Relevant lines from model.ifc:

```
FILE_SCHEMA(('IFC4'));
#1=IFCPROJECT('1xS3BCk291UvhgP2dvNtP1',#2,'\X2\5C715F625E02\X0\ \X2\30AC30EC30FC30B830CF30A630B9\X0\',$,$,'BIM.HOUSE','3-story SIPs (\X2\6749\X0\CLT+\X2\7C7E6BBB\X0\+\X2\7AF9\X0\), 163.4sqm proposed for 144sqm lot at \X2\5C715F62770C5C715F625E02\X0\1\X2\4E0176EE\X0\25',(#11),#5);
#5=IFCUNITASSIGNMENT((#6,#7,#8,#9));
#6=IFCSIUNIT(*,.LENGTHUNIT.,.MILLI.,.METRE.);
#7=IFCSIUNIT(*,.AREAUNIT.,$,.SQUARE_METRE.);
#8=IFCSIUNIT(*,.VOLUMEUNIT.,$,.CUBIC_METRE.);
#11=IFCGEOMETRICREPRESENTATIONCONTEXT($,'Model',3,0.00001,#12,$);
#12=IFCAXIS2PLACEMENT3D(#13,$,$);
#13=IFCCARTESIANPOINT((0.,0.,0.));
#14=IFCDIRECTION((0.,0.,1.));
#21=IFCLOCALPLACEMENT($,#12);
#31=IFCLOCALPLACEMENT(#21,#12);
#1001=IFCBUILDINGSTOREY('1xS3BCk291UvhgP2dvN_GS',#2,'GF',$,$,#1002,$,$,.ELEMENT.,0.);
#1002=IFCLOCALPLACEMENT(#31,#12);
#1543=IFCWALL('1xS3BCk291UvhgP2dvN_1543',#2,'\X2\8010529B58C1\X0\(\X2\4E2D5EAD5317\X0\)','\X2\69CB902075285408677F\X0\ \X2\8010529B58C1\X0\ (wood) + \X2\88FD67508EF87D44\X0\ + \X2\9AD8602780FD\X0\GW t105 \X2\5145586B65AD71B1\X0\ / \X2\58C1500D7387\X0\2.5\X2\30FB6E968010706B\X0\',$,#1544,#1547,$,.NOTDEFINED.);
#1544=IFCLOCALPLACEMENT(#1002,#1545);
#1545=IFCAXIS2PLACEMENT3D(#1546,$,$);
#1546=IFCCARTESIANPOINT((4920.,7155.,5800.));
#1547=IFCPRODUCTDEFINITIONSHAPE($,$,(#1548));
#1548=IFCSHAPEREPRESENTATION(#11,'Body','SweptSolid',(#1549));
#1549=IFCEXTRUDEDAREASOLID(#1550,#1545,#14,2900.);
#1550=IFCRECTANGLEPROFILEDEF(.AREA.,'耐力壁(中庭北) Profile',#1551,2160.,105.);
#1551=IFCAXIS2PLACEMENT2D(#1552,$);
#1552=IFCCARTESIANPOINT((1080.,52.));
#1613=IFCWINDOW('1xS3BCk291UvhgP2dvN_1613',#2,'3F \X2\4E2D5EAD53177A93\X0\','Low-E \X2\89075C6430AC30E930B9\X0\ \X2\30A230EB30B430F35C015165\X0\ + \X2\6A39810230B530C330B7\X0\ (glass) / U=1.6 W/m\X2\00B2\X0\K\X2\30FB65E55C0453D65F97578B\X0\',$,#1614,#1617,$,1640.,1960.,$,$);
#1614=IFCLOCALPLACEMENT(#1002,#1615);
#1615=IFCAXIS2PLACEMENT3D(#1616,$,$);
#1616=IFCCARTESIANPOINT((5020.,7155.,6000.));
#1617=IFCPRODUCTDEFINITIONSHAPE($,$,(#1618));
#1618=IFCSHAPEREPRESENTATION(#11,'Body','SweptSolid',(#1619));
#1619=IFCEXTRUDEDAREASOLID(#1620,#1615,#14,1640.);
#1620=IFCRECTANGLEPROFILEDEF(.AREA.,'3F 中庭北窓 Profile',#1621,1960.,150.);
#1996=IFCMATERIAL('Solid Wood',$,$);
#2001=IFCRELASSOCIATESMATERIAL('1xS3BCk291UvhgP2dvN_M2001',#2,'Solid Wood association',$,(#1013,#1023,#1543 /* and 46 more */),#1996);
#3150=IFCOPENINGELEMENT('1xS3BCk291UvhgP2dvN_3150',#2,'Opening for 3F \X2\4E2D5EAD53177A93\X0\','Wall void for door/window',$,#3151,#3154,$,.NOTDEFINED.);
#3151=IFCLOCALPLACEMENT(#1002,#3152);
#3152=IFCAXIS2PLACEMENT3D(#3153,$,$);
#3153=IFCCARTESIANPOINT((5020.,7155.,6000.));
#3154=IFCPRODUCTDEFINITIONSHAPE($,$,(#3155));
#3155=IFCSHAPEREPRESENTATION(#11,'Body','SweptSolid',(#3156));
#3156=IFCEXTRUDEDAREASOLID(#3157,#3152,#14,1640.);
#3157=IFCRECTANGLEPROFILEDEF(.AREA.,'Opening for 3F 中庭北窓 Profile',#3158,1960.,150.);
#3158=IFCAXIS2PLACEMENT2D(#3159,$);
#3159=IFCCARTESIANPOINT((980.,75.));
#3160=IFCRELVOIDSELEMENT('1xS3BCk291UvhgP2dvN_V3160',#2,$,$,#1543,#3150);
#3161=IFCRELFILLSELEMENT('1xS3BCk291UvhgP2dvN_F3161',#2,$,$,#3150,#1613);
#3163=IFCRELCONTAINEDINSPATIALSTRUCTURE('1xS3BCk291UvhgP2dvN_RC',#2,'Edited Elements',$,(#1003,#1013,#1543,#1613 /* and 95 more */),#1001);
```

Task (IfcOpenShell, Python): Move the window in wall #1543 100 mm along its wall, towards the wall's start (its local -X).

```python
import ifcopenshell
import ifcopenshell.api.geometry
import ifcopenshell.util.placement
import ifcopenshell.util.unit

model = ifcopenshell.open("model.ifc")
unit_scale = ifcopenshell.util.unit.calculate_unit_scale(model)

window = model.by_guid("1xS3BCk291UvhgP2dvN_1613")
opening = window.FillsVoids[0].RelatingOpeningElement
wall = opening.VoidsElements[0].RelatingBuildingElement

wall_matrix = ifcopenshell.util.placement.get_local_placement(wall.ObjectPlacement)
shift = wall_matrix[:3, 0] * -0.1 / unit_scale
before = ifcopenshell.util.placement.get_local_placement(window.ObjectPlacement)[:3, 3].copy()

# The window is not placed relative to its opening, so move both.
for product in (opening, window):
    matrix = ifcopenshell.util.placement.get_local_placement(product.ObjectPlacement)
    matrix[:3, 3] += shift
    ifcopenshell.api.geometry.edit_object_placement(model, product=product, matrix=matrix, is_si=False)

after = ifcopenshell.util.placement.get_local_placement(window.ObjectPlacement)[:3, 3]
print("window moved by", (after - before).round(3) + 0.0)

model.write("model-out.ifc")
```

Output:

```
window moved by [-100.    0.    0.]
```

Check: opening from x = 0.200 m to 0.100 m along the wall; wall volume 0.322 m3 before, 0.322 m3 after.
